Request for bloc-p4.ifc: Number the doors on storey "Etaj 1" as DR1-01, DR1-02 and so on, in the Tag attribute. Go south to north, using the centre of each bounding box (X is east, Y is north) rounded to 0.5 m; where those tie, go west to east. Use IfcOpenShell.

First a look at what the model holds.

```python
import ifcopenshell
import ifcopenshell.util.element
import ifcopenshell.util.placement

model = ifcopenshell.open("bloc-p4.ifc")
print(model.schema)
storey = next(s for s in model.by_type("IfcBuildingStorey") if s.Name == "Etaj 1")
doors = [e for e in ifcopenshell.util.element.get_decomposition(storey) if e.is_a("IfcDoor")]
for e in sorted(doors, key=lambda e: e.id()):
    origin = ifcopenshell.util.placement.get_local_placement(e.ObjectPlacement)[:3, 3]
    print(e.id(), e.Tag, e.Name, origin.round(2) + 0.0, sep=" | ")
```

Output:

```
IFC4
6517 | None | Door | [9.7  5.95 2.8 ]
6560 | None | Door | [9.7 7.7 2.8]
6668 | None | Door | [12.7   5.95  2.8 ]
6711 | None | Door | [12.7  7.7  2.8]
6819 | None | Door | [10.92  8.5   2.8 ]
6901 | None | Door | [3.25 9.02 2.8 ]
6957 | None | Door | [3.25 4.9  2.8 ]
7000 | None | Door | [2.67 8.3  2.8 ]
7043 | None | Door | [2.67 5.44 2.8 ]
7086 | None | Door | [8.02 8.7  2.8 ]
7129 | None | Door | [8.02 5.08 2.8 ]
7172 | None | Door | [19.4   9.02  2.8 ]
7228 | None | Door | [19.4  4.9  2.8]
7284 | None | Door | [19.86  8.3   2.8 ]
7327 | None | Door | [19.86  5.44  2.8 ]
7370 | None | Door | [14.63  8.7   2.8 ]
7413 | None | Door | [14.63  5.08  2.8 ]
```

```python
import ifcopenshell
import ifcopenshell.geom
import ifcopenshell.util.element
import ifcopenshell.util.shape

model = ifcopenshell.open("bloc-p4.ifc")
settings = ifcopenshell.geom.settings()
settings.set("use-world-coords", True)


def centre(element):
    shape = ifcopenshell.geom.create_shape(settings, element)
    return ifcopenshell.util.shape.get_bbox_centroid(shape.geometry)


storey = next(s for s in model.by_type("IfcBuildingStorey") if s.Name == "Etaj 1")
doors = [e for e in ifcopenshell.util.element.get_decomposition(storey) if e.is_a("IfcDoor")]

# Insertion points can sit at a corner or the storey origin, so sort by the geometry (in metres).
centres = {e: centre(e) for e in doors}
doors.sort(key=lambda e: (round(centres[e][1] / 0.5), centres[e][0]))

for i, e in enumerate(doors, start=1):
    number = f"DR1-{i:02d}"
    e.Tag = number
    print(e.id(), number)

model.write("bloc-p4-out.ifc")
```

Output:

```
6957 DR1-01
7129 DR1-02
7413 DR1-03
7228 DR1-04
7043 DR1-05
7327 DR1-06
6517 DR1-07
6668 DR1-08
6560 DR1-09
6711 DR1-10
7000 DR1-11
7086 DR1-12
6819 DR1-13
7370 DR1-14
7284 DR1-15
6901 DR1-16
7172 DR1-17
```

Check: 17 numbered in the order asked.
